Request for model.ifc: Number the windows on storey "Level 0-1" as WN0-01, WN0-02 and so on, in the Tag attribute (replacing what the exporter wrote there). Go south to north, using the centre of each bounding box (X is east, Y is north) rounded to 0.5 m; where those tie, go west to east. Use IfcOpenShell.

First a look at what the model holds.

```python
import ifcopenshell
import ifcopenshell.util.element
import ifcopenshell.util.placement

model = ifcopenshell.open("model.ifc")
print(model.schema)
storey = next(s for s in model.by_type("IfcBuildingStorey") if s.Name == "Level 0-1")
windows = [e for e in ifcopenshell.util.element.get_decomposition(storey) if e.is_a("IfcWindow")]
for e in sorted(windows, key=lambda e: e.id()):
    origin = ifcopenshell.util.placement.get_local_placement(e.ObjectPlacement)[:3, 3]
    print(e.id(), e.Tag, e.Name, origin.round(2) + 0.0, sep=" | ")
```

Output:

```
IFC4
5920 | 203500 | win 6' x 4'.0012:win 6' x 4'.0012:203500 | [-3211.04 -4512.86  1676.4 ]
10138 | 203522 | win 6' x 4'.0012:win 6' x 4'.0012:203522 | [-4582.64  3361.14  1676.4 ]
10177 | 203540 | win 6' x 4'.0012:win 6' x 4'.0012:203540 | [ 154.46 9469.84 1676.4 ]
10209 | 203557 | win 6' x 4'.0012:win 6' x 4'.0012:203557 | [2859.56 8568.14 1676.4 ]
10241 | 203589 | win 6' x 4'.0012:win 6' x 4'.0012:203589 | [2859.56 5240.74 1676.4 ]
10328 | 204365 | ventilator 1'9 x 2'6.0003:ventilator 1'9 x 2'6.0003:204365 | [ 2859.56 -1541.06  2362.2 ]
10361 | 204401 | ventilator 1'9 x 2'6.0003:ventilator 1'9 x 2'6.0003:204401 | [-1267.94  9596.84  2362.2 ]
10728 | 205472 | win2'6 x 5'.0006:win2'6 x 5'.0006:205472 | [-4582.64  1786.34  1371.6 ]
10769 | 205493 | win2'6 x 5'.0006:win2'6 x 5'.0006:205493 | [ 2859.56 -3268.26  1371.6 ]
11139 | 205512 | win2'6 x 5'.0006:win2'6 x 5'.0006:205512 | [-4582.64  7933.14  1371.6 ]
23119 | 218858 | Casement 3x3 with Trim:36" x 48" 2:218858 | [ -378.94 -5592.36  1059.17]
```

```python
import ifcopenshell
import ifcopenshell.geom
import ifcopenshell.util.element
import ifcopenshell.util.shape

model = ifcopenshell.open("model.ifc")
settings = ifcopenshell.geom.settings()
settings.set("use-world-coords", True)


def centre(element):
    shape = ifcopenshell.geom.create_shape(settings, element)
    return ifcopenshell.util.shape.get_bbox_centroid(shape.geometry)


storey = next(s for s in model.by_type("IfcBuildingStorey") if s.Name == "Level 0-1")
windows = [e for e in ifcopenshell.util.element.get_decomposition(storey) if e.is_a("IfcWindow")]

# Insertion points can sit at a corner or the storey origin, so sort by the geometry (in metres).
centres = {e: centre(e) for e in windows}
windows.sort(key=lambda e: (round(centres[e][1] / 0.5), centres[e][0]))

for i, e in enumerate(windows, start=1):
    number = f"WN0-{i:02d}"
    e.Tag = number
    print(e.id(), number)

model.write("model_rev.ifc")
```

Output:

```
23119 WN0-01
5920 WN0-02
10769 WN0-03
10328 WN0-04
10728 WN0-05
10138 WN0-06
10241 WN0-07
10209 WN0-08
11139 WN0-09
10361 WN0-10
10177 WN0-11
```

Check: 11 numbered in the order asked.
